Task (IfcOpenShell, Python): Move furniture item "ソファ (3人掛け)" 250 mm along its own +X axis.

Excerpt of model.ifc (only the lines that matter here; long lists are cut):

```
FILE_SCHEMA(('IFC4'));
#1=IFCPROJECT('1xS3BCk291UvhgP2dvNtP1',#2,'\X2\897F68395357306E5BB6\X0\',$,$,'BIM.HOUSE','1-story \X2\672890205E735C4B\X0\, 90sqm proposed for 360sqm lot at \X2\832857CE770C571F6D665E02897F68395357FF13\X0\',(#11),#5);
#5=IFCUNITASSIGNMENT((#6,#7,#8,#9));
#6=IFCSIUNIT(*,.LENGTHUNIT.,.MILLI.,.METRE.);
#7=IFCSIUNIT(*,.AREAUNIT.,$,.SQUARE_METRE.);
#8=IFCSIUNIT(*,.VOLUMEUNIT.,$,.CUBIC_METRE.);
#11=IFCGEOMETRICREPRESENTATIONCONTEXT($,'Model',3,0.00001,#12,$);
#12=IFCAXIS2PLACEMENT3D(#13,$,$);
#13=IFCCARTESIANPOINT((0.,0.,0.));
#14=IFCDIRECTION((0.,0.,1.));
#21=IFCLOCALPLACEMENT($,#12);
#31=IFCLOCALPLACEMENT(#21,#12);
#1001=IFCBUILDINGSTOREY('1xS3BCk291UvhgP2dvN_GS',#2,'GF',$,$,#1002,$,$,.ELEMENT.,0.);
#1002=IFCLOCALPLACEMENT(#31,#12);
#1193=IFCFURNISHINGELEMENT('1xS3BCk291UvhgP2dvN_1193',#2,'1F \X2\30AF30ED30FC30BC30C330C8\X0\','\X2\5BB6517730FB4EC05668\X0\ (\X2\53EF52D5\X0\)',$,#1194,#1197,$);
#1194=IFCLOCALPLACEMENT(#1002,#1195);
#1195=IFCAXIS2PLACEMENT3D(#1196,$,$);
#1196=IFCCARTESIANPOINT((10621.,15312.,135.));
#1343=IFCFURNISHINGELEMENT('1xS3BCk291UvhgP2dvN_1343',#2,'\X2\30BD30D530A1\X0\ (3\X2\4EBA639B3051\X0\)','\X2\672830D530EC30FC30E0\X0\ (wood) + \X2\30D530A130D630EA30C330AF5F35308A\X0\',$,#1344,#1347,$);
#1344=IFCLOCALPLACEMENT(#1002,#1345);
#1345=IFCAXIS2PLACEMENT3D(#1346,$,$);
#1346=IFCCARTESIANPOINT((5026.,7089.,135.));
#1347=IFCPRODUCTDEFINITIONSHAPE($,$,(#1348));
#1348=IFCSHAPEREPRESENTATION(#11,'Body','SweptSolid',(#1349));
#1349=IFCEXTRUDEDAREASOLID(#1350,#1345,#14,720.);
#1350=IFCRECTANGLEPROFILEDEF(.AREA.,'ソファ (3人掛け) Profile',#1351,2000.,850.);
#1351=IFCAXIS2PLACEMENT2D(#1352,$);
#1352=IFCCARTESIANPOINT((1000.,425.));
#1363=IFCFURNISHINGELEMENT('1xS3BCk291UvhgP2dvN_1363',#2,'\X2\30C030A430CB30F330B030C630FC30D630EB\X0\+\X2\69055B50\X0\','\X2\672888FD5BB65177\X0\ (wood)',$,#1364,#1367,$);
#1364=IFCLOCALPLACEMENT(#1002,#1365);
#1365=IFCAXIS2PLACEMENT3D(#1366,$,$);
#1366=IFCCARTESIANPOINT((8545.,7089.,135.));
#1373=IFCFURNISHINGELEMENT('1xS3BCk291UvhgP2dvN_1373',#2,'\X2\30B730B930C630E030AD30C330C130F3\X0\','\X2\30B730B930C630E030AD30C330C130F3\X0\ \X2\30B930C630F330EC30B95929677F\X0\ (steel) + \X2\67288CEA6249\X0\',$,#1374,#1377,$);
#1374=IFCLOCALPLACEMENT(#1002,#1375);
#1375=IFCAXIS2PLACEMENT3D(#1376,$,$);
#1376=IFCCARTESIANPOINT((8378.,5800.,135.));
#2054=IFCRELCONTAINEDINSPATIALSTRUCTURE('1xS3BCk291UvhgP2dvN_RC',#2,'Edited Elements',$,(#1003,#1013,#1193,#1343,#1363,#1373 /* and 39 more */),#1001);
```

```python
import ifcopenshell
import ifcopenshell.api.geometry
import ifcopenshell.util.placement
import ifcopenshell.util.unit

model = ifcopenshell.open("model.ifc")
unit_scale = ifcopenshell.util.unit.calculate_unit_scale(model)

item = model.by_id(1343)
matrix = ifcopenshell.util.placement.get_local_placement(item.ObjectPlacement)
matrix[:3, 3] += matrix[:3, 0] * 0.25 / unit_scale
ifcopenshell.api.geometry.edit_object_placement(model, product=item, matrix=matrix, is_si=False)

print(ifcopenshell.util.placement.get_local_placement(item.ObjectPlacement).round(3) + 0.0)

model.write("model_rev.ifc")
```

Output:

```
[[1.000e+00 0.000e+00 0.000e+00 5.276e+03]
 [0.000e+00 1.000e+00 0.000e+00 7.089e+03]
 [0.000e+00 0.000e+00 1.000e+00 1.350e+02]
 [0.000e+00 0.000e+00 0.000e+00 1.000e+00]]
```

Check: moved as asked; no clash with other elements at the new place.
